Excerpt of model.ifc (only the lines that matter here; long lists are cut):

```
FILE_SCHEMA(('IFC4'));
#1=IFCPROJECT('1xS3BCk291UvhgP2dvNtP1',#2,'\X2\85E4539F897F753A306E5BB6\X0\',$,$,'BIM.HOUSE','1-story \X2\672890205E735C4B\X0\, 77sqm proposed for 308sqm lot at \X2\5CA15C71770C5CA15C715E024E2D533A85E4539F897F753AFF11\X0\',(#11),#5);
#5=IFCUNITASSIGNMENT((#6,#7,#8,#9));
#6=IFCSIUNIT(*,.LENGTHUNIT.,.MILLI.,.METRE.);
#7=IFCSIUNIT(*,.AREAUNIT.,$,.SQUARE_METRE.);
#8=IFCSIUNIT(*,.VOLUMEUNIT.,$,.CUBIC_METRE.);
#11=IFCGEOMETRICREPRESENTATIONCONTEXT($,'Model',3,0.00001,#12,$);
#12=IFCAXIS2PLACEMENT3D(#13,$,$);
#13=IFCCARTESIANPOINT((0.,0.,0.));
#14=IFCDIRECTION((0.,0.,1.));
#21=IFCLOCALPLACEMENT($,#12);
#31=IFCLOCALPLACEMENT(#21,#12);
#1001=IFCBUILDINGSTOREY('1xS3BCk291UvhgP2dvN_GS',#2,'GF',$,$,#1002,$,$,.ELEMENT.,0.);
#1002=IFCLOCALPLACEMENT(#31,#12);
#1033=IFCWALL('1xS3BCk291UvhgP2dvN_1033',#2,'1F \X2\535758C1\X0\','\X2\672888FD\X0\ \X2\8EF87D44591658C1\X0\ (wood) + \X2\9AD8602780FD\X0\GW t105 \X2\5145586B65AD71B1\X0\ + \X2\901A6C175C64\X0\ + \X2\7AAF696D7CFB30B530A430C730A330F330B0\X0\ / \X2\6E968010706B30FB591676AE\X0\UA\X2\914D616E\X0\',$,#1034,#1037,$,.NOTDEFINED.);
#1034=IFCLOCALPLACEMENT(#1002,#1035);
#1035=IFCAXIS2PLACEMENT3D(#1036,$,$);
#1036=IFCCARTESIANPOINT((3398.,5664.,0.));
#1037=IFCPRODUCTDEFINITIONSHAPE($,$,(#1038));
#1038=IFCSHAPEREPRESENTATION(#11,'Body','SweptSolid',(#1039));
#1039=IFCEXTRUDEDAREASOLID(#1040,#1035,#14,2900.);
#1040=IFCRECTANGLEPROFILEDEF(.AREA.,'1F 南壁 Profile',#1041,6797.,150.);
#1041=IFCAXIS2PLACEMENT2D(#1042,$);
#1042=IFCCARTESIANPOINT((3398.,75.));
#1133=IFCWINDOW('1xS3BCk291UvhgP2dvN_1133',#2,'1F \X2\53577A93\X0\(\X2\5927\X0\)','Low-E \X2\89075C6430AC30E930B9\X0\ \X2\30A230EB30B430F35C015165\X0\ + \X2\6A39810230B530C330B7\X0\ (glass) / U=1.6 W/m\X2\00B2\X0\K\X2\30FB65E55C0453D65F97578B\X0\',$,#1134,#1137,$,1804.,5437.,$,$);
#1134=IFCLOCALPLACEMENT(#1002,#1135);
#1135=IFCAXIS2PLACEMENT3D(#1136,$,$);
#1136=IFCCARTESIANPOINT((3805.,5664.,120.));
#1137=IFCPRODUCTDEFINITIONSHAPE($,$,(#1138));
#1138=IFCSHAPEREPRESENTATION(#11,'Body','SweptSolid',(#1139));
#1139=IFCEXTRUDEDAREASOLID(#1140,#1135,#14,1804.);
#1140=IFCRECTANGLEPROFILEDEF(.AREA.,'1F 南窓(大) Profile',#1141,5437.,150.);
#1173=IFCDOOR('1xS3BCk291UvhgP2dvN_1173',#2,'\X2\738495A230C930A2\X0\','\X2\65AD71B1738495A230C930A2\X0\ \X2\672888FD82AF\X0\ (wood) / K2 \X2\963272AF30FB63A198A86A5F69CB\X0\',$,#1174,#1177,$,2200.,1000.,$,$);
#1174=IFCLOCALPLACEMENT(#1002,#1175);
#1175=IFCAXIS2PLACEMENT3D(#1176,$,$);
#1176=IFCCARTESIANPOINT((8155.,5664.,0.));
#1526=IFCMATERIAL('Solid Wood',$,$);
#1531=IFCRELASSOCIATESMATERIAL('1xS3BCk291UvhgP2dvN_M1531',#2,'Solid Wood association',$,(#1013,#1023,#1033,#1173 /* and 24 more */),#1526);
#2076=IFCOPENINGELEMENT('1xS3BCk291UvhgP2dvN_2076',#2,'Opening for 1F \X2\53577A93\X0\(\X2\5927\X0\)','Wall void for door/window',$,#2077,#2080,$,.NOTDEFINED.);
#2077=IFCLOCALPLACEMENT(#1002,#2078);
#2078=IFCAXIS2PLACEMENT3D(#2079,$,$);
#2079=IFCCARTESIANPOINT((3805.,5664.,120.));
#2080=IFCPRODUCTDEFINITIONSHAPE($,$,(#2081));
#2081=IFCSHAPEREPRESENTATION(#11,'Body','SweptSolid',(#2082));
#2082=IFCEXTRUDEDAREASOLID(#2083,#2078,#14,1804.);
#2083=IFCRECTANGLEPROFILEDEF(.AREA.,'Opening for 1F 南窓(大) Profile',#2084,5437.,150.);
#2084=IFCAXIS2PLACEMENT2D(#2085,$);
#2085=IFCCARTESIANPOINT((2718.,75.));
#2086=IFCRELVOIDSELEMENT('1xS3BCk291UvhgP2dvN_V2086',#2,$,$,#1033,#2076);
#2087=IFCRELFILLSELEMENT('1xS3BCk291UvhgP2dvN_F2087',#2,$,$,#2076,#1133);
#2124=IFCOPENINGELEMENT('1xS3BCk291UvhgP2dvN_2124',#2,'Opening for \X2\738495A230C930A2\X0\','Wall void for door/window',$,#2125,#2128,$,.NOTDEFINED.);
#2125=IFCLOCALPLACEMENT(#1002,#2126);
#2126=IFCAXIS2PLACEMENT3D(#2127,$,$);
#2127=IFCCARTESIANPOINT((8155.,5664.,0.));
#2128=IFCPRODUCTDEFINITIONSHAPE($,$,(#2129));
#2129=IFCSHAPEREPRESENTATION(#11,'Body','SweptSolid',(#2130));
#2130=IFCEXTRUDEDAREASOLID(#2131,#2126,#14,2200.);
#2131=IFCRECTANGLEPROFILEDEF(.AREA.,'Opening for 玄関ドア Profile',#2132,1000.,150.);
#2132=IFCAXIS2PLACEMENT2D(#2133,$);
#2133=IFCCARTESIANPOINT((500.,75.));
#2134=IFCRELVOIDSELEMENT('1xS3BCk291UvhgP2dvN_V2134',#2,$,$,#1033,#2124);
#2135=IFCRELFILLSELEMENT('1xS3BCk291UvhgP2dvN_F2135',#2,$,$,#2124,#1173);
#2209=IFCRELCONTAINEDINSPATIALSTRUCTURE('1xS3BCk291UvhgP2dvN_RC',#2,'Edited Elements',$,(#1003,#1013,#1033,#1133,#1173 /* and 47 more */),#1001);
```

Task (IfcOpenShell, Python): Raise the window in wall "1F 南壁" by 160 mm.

```python
import numpy as np
import ifcopenshell
import ifcopenshell.api.geometry
import ifcopenshell.util.placement
import ifcopenshell.util.unit

model = ifcopenshell.open("model.ifc")
unit_scale = ifcopenshell.util.unit.calculate_unit_scale(model)

window = model.by_guid("1xS3BCk291UvhgP2dvN_1133")
opening = window.FillsVoids[0].RelatingOpeningElement
dz = 160.0

shift = np.array([0.0, 0.0, dz])
# The window is not placed relative to its opening, so move both.
for product in (opening, window):
    matrix = ifcopenshell.util.placement.get_local_placement(product.ObjectPlacement)
    matrix[:3, 3] += shift
    ifcopenshell.api.geometry.edit_object_placement(model, product=product, matrix=matrix, is_si=False)

print(f"moved by {dz * unit_scale:+.3f} m")

model.write("model_edited.ifc")
```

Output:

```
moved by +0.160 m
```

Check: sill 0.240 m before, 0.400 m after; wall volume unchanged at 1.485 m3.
